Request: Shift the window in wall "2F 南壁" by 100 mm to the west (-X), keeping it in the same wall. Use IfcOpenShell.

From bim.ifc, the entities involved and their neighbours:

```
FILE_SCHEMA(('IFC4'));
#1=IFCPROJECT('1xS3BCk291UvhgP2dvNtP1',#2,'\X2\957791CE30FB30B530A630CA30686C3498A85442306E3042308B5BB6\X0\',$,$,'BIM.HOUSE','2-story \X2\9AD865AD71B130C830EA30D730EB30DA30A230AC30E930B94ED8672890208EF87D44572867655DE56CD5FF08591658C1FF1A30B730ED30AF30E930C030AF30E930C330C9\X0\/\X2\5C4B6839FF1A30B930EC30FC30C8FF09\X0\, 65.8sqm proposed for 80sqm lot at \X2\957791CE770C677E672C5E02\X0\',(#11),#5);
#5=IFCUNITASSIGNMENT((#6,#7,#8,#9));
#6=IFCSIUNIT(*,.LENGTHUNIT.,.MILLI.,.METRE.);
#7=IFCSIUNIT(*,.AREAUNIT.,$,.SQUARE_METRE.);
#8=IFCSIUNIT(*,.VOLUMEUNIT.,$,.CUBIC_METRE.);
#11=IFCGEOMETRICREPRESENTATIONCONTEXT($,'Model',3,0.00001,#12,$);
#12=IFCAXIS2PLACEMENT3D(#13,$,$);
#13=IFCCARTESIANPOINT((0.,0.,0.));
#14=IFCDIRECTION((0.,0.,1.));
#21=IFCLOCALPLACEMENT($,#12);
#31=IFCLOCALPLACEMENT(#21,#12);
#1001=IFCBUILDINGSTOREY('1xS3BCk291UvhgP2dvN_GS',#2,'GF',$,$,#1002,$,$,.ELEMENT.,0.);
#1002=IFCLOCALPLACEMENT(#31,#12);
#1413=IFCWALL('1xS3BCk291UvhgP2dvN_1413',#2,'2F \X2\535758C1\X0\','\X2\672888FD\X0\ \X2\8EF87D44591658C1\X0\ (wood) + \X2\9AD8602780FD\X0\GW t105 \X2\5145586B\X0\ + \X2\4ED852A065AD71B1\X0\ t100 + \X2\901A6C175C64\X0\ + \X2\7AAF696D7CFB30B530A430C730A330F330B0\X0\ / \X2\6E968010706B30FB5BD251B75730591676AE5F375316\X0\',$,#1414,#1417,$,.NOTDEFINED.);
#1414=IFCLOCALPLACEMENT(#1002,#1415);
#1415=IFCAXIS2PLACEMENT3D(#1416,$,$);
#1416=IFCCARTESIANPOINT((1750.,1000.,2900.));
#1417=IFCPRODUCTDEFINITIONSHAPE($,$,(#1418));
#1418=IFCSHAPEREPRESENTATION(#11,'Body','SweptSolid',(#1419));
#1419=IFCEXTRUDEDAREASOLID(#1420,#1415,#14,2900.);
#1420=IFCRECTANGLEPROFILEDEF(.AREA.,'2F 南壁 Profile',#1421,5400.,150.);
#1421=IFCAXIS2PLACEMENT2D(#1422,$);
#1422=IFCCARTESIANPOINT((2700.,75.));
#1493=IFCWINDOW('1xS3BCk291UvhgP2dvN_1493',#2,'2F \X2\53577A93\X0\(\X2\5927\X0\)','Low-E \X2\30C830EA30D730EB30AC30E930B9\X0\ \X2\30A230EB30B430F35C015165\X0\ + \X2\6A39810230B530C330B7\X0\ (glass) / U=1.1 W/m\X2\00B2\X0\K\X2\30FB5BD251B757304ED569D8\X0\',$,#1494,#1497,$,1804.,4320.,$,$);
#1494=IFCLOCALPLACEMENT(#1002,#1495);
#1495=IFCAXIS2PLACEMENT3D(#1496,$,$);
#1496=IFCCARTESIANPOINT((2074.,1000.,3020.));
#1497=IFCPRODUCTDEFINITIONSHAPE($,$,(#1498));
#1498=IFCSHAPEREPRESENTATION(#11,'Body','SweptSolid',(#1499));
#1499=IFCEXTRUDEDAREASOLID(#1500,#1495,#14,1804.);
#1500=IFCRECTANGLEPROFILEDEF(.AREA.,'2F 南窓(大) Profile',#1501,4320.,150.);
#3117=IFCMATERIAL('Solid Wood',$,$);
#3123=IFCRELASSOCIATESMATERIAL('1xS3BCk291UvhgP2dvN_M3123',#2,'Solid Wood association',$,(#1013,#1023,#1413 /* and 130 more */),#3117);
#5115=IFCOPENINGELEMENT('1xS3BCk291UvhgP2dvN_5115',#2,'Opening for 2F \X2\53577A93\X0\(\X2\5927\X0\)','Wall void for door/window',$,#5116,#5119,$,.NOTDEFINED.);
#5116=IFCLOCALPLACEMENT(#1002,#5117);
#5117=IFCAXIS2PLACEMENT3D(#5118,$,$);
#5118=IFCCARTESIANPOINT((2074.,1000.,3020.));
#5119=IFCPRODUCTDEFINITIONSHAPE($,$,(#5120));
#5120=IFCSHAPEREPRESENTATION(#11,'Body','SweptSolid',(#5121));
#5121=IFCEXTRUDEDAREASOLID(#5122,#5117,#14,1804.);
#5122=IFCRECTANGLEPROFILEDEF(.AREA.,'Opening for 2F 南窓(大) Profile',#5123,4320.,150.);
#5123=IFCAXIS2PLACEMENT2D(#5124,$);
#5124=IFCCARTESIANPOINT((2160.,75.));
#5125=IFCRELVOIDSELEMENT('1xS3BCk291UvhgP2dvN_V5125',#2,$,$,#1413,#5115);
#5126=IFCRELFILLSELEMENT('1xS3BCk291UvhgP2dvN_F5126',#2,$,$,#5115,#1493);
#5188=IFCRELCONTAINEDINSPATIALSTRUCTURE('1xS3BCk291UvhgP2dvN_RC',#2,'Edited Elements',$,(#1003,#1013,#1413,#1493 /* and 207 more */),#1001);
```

```python
import ifcopenshell
import ifcopenshell.api.geometry
import ifcopenshell.util.placement
import ifcopenshell.util.unit

model = ifcopenshell.open("bim.ifc")
unit_scale = ifcopenshell.util.unit.calculate_unit_scale(model)

window = model.by_id(1493)
opening = window.FillsVoids[0].RelatingOpeningElement
wall = opening.VoidsElements[0].RelatingBuildingElement

wall_matrix = ifcopenshell.util.placement.get_local_placement(wall.ObjectPlacement)
shift = wall_matrix[:3, 0] * -0.1 / unit_scale
before = ifcopenshell.util.placement.get_local_placement(window.ObjectPlacement)[:3, 3].copy()

# The window is not placed relative to its opening, so move both.
for product in (opening, window):
    matrix = ifcopenshell.util.placement.get_local_placement(product.ObjectPlacement)
    matrix[:3, 3] += shift
    ifcopenshell.api.geometry.edit_object_placement(model, product=product, matrix=matrix, is_si=False)

after = ifcopenshell.util.placement.get_local_placement(window.ObjectPlacement)[:3, 3]
print("window moved by", (after - before).round(3) + 0.0)

model.write("bim-out.ifc")
```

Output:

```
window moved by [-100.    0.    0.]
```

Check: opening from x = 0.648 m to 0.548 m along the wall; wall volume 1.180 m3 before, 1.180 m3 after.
